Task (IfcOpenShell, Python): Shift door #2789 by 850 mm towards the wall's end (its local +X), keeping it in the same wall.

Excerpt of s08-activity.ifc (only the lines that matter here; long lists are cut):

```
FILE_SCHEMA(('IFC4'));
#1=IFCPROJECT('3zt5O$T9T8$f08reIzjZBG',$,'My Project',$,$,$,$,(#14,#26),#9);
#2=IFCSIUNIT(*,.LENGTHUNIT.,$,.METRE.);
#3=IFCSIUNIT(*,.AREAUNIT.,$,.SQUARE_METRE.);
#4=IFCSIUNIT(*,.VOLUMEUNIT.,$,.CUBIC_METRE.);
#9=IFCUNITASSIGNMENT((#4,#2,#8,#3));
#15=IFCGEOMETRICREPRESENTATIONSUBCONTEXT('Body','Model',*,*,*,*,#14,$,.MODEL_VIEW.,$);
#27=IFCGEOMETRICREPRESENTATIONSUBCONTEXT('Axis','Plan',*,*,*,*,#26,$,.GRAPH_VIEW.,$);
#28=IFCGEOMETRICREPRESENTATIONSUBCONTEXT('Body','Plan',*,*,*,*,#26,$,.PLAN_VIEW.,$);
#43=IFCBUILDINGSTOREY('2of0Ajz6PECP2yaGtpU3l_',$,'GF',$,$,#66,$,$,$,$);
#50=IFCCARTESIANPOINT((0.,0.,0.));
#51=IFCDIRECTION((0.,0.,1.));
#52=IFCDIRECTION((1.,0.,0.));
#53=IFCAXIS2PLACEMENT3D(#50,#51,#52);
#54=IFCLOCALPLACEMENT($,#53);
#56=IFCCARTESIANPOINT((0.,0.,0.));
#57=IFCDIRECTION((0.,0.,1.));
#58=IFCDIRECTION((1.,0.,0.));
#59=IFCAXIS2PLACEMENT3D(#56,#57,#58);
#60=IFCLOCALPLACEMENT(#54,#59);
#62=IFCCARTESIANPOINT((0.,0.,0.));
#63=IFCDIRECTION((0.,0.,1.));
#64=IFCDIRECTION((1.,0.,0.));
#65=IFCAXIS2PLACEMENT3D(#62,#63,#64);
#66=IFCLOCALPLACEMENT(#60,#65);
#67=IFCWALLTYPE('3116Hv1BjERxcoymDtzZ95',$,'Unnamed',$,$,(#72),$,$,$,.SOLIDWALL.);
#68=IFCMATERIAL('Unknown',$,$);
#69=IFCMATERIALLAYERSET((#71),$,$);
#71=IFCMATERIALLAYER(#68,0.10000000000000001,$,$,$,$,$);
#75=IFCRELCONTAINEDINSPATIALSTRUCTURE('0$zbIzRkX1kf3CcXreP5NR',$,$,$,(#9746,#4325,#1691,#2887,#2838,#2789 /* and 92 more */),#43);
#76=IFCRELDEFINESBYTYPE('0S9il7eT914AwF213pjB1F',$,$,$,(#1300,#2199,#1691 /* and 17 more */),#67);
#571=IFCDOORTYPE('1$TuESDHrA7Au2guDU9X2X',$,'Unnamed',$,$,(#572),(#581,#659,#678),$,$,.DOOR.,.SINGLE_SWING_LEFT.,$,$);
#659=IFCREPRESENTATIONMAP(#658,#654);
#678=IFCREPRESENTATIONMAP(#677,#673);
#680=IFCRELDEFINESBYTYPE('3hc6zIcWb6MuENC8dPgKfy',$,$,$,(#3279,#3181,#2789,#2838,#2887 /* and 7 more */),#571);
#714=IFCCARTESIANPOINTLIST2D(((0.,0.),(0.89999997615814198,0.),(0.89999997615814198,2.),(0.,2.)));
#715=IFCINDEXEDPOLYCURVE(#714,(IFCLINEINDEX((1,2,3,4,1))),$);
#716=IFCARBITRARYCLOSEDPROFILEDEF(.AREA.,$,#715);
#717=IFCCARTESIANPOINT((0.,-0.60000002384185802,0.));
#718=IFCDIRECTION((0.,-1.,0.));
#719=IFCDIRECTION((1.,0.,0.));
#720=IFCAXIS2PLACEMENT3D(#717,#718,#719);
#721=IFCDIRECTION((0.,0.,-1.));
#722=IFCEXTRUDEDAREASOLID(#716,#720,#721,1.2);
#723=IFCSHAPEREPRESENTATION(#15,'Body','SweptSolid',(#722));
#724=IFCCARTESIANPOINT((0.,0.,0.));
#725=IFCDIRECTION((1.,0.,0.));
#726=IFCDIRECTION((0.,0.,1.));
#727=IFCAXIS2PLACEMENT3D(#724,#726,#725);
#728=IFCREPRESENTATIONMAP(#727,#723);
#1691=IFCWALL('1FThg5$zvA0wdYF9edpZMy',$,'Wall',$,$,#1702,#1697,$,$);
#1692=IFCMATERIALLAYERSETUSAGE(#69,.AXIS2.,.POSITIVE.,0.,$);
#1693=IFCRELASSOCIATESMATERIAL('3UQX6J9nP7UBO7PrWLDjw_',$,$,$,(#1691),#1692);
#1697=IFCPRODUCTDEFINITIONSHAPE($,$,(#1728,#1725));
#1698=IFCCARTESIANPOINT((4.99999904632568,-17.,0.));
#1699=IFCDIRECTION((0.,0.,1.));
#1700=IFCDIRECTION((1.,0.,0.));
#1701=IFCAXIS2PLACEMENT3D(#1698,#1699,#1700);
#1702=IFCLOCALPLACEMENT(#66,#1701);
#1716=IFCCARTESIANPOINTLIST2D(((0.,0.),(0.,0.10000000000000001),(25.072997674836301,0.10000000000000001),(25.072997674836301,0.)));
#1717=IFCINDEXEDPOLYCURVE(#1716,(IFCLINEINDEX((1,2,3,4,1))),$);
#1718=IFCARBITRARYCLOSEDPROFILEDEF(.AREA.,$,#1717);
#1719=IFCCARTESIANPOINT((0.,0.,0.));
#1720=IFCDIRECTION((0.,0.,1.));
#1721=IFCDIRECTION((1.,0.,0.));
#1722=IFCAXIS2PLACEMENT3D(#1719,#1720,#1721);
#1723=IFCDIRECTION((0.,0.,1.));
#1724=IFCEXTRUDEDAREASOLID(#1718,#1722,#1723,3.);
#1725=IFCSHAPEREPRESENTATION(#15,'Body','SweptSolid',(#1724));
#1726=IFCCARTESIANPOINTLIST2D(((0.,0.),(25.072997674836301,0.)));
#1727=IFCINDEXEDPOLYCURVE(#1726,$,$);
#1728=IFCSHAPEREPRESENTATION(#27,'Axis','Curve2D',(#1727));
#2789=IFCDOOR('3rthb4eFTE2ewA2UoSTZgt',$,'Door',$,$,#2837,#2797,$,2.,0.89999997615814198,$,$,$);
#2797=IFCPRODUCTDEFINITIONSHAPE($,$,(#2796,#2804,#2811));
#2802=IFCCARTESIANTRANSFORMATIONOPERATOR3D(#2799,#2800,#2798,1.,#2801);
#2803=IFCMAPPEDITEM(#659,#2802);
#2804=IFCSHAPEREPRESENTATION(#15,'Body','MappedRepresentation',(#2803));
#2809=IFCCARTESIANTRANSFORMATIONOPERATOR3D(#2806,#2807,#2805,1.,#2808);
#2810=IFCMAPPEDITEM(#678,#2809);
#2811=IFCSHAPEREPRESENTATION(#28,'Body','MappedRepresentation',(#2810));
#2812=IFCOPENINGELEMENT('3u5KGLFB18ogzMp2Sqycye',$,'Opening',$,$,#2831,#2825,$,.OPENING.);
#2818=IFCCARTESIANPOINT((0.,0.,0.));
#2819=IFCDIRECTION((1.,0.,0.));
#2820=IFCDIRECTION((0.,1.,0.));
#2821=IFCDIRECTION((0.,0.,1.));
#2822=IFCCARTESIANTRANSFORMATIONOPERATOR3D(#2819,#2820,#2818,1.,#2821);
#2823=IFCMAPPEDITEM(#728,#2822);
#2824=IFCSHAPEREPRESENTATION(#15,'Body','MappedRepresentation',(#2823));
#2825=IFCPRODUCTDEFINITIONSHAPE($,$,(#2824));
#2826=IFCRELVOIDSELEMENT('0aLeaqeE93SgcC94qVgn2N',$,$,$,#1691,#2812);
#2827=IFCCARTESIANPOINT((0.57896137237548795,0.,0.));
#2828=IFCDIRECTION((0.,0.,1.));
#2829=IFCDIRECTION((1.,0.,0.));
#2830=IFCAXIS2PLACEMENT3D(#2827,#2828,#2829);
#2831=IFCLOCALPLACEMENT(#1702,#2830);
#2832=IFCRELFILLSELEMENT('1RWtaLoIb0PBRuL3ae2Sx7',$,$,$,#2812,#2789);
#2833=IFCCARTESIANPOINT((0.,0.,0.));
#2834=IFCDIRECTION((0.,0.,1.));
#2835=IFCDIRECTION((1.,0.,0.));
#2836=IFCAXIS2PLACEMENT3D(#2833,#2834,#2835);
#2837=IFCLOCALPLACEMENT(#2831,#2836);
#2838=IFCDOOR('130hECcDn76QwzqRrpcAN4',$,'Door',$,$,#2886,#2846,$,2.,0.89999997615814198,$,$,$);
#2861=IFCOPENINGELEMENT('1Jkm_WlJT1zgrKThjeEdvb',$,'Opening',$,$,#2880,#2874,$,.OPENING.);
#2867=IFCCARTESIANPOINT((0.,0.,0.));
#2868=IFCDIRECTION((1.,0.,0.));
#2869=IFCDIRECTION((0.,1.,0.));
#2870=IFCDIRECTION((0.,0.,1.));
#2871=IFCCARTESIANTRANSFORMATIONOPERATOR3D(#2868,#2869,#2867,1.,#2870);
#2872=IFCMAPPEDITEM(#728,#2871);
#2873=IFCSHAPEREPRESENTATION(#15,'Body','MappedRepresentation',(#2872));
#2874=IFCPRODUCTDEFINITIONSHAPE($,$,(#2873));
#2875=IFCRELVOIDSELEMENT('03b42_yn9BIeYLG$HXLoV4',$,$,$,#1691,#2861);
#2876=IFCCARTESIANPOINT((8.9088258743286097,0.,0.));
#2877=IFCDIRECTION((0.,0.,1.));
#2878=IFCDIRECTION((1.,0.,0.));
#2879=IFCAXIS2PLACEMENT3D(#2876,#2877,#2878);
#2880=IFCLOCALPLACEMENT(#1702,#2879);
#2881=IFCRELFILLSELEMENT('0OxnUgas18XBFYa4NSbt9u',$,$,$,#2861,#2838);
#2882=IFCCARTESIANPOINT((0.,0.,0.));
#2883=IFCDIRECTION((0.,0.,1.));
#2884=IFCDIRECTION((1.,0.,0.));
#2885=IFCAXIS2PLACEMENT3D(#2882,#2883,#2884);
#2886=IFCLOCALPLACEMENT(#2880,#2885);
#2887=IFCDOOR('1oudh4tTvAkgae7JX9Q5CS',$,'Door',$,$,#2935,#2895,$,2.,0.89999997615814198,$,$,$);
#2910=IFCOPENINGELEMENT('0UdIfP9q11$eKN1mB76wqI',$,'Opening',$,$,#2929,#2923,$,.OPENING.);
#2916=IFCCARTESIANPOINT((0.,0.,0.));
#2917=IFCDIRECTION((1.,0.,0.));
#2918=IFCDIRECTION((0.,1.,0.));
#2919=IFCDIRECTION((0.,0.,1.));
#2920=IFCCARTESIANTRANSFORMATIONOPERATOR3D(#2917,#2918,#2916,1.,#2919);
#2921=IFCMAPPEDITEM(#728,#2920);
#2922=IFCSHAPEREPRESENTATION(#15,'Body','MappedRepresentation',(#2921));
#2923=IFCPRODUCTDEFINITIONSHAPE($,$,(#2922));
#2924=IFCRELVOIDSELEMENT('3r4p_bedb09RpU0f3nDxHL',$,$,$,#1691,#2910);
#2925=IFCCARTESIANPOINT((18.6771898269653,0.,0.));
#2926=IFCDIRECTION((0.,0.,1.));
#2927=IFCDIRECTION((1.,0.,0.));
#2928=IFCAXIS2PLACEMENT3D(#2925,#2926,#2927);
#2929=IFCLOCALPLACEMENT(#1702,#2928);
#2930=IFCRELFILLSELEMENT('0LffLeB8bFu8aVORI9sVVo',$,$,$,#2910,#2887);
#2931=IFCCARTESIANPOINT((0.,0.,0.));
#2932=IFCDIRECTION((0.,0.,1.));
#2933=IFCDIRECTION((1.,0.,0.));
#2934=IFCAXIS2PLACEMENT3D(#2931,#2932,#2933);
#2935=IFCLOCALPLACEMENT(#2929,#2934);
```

```python
import ifcopenshell
import ifcopenshell.api.geometry
import ifcopenshell.util.placement
import ifcopenshell.util.unit

model = ifcopenshell.open("s08-activity.ifc")
unit_scale = ifcopenshell.util.unit.calculate_unit_scale(model)

door = model.by_id(2789)
opening = door.FillsVoids[0].RelatingOpeningElement
wall = opening.VoidsElements[0].RelatingBuildingElement

wall_matrix = ifcopenshell.util.placement.get_local_placement(wall.ObjectPlacement)
shift = wall_matrix[:3, 0] * 0.85 / unit_scale
before = ifcopenshell.util.placement.get_local_placement(door.ObjectPlacement)[:3, 3].copy()

# The door is placed relative to its opening, so it follows when the opening moves.
matrix = ifcopenshell.util.placement.get_local_placement(opening.ObjectPlacement)
matrix[:3, 3] += shift
ifcopenshell.api.geometry.edit_object_placement(
    model, product=opening, matrix=matrix, is_si=False, should_transform_children=True
)

after = ifcopenshell.util.placement.get_local_placement(door.ObjectPlacement)[:3, 3]
print("door moved by", (after - before).round(3) + 0.0)

model.write("s08-activity-out.ifc")
```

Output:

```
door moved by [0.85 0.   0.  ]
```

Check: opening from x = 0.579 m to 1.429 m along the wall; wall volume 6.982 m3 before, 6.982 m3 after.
